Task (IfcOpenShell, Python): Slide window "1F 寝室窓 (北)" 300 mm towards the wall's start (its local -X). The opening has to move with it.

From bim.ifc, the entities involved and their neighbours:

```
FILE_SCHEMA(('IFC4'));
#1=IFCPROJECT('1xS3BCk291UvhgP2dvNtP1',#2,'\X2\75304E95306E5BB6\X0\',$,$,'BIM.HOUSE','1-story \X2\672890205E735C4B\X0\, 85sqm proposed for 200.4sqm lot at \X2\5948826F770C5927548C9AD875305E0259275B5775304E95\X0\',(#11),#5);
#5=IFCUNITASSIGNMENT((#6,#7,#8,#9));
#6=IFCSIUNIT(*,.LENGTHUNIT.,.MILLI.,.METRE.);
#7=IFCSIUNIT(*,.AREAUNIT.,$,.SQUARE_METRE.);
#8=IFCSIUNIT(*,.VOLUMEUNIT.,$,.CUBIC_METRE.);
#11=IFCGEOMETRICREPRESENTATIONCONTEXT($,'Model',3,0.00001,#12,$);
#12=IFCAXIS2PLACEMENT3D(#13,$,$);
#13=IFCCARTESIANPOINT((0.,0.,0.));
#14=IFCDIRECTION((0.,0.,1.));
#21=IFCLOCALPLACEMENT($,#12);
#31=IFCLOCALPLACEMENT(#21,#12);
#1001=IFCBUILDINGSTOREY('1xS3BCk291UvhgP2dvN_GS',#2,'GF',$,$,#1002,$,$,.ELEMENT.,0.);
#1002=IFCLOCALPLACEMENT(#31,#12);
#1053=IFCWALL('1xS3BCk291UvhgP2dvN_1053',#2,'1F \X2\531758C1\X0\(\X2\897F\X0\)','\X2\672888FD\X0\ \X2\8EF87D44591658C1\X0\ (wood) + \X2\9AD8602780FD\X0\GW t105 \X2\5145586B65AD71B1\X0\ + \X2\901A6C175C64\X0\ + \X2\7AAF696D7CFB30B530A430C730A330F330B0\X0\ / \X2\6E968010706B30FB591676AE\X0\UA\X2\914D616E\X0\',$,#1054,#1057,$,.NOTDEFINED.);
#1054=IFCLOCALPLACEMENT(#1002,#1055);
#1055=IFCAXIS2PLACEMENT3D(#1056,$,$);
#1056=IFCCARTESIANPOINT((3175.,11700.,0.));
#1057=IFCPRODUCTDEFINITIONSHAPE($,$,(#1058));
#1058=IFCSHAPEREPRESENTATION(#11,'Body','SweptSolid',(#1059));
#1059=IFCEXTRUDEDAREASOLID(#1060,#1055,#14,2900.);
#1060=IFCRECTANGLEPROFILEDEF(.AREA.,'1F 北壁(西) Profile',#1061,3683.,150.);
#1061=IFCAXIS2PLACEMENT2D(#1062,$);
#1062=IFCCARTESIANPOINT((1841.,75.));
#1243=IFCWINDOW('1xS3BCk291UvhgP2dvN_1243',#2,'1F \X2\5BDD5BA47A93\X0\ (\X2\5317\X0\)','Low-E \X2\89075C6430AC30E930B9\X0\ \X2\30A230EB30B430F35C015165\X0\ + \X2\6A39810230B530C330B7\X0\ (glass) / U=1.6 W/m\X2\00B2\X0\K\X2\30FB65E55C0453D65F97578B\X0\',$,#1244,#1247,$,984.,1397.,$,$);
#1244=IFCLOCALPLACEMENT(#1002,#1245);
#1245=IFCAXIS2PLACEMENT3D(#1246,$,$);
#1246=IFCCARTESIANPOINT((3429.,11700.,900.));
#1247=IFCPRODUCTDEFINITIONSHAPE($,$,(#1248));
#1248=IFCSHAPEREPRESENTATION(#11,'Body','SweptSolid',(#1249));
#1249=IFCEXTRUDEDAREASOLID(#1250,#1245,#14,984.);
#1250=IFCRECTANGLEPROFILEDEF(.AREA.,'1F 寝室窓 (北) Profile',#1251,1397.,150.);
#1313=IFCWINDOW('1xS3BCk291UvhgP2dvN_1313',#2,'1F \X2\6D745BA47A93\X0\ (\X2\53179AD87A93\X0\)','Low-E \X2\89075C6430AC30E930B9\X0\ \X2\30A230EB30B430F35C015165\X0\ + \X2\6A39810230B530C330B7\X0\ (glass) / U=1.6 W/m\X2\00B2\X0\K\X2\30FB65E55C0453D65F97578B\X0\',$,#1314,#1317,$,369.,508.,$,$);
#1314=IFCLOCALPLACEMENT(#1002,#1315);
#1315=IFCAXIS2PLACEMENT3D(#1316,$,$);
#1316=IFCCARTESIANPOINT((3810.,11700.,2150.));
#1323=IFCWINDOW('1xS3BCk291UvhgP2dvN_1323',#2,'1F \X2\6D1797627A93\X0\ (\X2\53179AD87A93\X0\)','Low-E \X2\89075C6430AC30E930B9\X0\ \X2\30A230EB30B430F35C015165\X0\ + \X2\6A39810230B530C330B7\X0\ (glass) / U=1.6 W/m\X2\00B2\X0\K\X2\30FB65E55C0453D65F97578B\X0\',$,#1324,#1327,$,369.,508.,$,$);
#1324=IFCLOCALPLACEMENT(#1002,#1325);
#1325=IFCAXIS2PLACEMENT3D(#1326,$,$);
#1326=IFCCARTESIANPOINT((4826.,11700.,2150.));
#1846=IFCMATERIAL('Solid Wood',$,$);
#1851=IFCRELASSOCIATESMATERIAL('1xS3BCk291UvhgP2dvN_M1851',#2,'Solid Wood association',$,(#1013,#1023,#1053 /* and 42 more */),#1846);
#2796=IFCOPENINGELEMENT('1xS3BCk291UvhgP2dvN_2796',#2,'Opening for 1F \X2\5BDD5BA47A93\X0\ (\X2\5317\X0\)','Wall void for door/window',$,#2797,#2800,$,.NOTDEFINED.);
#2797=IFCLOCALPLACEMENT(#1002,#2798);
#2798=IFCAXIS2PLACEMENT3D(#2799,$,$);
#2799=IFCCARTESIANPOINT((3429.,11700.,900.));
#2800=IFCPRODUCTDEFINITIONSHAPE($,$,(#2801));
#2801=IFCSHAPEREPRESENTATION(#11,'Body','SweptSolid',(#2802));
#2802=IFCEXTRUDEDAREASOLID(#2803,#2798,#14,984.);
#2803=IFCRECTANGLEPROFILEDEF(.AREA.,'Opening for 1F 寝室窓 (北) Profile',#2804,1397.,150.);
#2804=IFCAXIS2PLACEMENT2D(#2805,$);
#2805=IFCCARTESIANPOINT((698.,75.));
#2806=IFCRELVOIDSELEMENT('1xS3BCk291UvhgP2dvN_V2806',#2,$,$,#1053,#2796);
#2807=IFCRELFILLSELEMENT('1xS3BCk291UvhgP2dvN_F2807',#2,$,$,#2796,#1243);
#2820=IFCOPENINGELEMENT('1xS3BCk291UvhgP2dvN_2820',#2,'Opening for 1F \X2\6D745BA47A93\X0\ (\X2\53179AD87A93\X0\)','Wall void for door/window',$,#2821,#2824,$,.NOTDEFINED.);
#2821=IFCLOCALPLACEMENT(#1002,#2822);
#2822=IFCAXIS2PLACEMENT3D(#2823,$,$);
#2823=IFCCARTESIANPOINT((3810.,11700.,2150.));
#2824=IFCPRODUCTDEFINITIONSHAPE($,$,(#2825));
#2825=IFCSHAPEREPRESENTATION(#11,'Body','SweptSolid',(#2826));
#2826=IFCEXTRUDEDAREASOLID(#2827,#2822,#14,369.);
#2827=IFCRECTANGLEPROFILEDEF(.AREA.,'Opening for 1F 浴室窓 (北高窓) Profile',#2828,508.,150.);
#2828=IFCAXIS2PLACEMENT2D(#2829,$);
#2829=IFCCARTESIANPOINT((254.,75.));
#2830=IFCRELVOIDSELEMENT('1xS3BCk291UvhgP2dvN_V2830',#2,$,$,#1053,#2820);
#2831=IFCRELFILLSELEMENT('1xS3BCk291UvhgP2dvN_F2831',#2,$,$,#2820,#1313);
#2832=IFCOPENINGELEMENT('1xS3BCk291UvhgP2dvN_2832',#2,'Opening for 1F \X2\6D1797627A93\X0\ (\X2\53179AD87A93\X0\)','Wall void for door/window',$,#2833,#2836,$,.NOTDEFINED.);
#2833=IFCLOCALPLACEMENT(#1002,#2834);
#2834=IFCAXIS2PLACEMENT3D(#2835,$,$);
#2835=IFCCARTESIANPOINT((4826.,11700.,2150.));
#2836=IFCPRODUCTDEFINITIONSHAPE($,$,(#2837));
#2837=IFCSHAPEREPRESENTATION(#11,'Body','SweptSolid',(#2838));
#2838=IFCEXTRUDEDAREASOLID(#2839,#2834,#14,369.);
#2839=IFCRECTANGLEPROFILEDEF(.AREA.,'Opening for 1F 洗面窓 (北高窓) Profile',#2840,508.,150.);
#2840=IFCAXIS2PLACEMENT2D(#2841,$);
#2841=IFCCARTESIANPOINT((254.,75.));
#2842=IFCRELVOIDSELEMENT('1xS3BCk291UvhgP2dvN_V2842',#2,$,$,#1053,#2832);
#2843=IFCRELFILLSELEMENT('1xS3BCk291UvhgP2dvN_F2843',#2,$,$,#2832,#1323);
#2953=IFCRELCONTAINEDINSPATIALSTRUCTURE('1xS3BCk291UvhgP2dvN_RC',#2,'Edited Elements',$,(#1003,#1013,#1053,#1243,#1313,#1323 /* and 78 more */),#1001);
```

```python
import ifcopenshell
import ifcopenshell.api.geometry
import ifcopenshell.util.placement
import ifcopenshell.util.unit

model = ifcopenshell.open("bim.ifc")
unit_scale = ifcopenshell.util.unit.calculate_unit_scale(model)

window = model.by_guid("1xS3BCk291UvhgP2dvN_1243")
opening = window.FillsVoids[0].RelatingOpeningElement
wall = opening.VoidsElements[0].RelatingBuildingElement

wall_matrix = ifcopenshell.util.placement.get_local_placement(wall.ObjectPlacement)
shift = wall_matrix[:3, 0] * -0.3 / unit_scale
before = ifcopenshell.util.placement.get_local_placement(window.ObjectPlacement)[:3, 3].copy()

# The window is not placed relative to its opening, so move both.
for product in (opening, window):
    matrix = ifcopenshell.util.placement.get_local_placement(product.ObjectPlacement)
    matrix[:3, 3] += shift
    ifcopenshell.api.geometry.edit_object_placement(model, product=product, matrix=matrix, is_si=False)

after = ifcopenshell.util.placement.get_local_placement(window.ObjectPlacement)[:3, 3]
print("window moved by", (after - before).round(3) + 0.0)

model.write("bim_updated.ifc")
```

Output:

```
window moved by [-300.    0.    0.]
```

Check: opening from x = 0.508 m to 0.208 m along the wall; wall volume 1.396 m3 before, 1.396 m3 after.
